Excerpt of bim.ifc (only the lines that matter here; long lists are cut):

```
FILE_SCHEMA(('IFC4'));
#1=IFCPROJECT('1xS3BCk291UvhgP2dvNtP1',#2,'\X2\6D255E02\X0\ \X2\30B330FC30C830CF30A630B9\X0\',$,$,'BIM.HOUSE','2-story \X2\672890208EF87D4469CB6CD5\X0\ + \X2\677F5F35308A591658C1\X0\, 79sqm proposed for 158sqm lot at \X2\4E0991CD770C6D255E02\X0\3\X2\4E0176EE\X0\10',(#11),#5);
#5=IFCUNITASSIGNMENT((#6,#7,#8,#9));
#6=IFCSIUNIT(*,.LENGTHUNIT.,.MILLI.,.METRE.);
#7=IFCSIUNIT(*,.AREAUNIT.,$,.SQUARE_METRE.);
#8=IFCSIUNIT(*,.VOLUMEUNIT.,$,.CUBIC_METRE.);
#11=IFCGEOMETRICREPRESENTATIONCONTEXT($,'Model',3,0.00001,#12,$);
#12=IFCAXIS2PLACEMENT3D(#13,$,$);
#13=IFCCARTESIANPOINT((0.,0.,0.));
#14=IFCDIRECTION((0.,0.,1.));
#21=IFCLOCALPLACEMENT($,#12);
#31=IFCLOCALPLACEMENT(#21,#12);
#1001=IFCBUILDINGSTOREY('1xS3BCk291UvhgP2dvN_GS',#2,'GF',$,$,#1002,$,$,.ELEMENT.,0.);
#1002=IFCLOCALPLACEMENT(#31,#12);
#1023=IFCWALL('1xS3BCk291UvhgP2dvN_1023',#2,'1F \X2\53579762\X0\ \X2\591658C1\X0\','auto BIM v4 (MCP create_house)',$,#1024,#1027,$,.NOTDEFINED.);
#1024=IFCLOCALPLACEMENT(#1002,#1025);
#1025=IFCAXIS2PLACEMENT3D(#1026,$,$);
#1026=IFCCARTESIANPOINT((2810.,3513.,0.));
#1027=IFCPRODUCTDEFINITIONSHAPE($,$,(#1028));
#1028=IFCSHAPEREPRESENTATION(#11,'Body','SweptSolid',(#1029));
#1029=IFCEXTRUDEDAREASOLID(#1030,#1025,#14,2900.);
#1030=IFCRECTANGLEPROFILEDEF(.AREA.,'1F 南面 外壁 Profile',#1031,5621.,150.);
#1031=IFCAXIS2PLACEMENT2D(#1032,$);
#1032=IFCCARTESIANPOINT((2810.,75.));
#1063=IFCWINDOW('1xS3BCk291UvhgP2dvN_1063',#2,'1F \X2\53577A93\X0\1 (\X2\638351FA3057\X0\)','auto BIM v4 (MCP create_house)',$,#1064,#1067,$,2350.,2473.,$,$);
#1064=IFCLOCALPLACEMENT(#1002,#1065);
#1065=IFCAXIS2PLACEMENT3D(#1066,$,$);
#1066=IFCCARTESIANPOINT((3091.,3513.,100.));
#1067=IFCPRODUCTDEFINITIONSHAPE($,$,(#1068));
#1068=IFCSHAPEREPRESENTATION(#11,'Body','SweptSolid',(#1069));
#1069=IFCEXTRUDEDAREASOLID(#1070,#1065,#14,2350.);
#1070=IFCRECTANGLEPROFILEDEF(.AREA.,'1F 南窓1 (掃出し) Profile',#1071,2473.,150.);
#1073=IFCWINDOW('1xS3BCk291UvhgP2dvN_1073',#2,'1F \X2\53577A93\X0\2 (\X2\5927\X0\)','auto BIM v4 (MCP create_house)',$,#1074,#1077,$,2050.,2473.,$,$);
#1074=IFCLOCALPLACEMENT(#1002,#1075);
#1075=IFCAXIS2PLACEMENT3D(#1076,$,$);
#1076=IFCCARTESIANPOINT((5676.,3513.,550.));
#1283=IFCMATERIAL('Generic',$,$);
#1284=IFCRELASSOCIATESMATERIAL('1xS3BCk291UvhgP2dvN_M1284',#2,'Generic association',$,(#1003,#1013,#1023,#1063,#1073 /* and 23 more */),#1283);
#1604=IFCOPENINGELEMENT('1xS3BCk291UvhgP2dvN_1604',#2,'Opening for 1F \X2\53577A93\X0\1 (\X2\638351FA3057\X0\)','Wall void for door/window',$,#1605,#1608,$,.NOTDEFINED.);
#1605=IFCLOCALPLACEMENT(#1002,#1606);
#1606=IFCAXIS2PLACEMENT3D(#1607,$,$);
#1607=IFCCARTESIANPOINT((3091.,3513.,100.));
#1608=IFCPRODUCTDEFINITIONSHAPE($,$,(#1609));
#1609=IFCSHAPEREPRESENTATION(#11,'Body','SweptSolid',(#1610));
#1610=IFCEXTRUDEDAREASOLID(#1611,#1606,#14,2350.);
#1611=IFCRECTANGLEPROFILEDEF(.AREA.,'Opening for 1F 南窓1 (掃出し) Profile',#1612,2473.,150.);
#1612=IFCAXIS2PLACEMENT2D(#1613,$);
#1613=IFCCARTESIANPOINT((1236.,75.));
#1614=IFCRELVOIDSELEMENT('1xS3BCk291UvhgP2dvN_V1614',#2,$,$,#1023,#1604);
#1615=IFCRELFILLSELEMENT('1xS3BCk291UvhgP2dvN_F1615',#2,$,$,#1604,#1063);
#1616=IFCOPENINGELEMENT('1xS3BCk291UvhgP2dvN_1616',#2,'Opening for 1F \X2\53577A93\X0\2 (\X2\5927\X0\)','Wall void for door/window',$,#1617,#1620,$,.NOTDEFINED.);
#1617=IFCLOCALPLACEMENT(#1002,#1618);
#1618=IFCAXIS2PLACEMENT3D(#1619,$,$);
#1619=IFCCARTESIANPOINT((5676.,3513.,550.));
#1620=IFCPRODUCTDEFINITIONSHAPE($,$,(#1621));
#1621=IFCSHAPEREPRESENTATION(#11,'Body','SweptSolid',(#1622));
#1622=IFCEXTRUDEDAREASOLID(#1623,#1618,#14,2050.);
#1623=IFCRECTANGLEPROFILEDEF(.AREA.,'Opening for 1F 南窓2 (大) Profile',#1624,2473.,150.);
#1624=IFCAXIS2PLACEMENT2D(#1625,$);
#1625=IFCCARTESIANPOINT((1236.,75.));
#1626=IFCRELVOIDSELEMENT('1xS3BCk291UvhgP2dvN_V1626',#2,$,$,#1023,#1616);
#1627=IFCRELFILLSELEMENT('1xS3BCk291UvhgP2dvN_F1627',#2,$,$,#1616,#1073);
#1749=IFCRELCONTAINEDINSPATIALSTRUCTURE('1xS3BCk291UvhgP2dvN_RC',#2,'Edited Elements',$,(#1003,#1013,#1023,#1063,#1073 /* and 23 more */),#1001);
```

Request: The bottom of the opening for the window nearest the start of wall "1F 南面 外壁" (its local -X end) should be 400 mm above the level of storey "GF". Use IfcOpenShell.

```python
import numpy as np
import ifcopenshell
import ifcopenshell.api.geometry
import ifcopenshell.geom
import ifcopenshell.util.element
import ifcopenshell.util.placement
import ifcopenshell.util.shape
import ifcopenshell.util.unit

model = ifcopenshell.open("bim.ifc")
unit_scale = ifcopenshell.util.unit.calculate_unit_scale(model)

window = model.by_guid("1xS3BCk291UvhgP2dvN_1063")
opening = window.FillsVoids[0].RelatingOpeningElement
storey = ifcopenshell.util.element.get_container(window, ifc_class="IfcBuildingStorey")
level = ifcopenshell.util.placement.get_local_placement(storey.ObjectPlacement)[2, 3]

# The opening's origin need not be at the sill, so measure its lowest point.
shape = ifcopenshell.geom.create_shape(ifcopenshell.geom.settings(), opening)
bottom = ifcopenshell.util.shape.get_shape_bottom_elevation(shape, shape.geometry) / unit_scale
dz = level + 0.4 / unit_scale - bottom

shift = np.array([0.0, 0.0, dz])
# The window is not placed relative to its opening, so move both.
for product in (opening, window):
    matrix = ifcopenshell.util.placement.get_local_placement(product.ObjectPlacement)
    matrix[:3, 3] += shift
    ifcopenshell.api.geometry.edit_object_placement(model, product=product, matrix=matrix, is_si=False)

print(f"moved by {dz * unit_scale:+.3f} m")

model.write("bim-out.ifc")
```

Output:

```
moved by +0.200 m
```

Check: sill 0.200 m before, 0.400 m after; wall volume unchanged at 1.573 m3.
